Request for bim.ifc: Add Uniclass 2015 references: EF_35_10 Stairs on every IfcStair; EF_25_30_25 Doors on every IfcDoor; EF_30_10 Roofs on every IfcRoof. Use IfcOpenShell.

First a look at what the model holds.

```python
import ifcopenshell

model = ifcopenshell.open("bim.ifc")
print(model.schema)
print("classifications:", [c.Name for c in model.by_type("IfcClassification")])
for ifc_class in ("IfcDoor", "IfcRoof", "IfcStair", "IfcWall", "IfcWindow"):
    print(ifc_class, len(model.by_type(ifc_class)))
```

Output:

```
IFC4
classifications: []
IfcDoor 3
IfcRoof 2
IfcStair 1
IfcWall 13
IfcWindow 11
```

```python
import ifcopenshell
import ifcopenshell.api.classification

model = ifcopenshell.open("bim.ifc")

system = ifcopenshell.api.classification.add_classification(model, classification="Uniclass 2015")

codes = {
    "IfcStair": ("EF_35_10", "Stairs"),
    "IfcDoor": ("EF_25_30_25", "Doors"),
    "IfcRoof": ("EF_30_10", "Roofs"),
}
for ifc_class, (code, name) in codes.items():
    products = model.by_type(ifc_class)
    ifcopenshell.api.classification.add_reference(
        model, products=products, classification=system, identification=code, name=name
    )
    print(code, len(products))

model.write("bim_edited.ifc")
```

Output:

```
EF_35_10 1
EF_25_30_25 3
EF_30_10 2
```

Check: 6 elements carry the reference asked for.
